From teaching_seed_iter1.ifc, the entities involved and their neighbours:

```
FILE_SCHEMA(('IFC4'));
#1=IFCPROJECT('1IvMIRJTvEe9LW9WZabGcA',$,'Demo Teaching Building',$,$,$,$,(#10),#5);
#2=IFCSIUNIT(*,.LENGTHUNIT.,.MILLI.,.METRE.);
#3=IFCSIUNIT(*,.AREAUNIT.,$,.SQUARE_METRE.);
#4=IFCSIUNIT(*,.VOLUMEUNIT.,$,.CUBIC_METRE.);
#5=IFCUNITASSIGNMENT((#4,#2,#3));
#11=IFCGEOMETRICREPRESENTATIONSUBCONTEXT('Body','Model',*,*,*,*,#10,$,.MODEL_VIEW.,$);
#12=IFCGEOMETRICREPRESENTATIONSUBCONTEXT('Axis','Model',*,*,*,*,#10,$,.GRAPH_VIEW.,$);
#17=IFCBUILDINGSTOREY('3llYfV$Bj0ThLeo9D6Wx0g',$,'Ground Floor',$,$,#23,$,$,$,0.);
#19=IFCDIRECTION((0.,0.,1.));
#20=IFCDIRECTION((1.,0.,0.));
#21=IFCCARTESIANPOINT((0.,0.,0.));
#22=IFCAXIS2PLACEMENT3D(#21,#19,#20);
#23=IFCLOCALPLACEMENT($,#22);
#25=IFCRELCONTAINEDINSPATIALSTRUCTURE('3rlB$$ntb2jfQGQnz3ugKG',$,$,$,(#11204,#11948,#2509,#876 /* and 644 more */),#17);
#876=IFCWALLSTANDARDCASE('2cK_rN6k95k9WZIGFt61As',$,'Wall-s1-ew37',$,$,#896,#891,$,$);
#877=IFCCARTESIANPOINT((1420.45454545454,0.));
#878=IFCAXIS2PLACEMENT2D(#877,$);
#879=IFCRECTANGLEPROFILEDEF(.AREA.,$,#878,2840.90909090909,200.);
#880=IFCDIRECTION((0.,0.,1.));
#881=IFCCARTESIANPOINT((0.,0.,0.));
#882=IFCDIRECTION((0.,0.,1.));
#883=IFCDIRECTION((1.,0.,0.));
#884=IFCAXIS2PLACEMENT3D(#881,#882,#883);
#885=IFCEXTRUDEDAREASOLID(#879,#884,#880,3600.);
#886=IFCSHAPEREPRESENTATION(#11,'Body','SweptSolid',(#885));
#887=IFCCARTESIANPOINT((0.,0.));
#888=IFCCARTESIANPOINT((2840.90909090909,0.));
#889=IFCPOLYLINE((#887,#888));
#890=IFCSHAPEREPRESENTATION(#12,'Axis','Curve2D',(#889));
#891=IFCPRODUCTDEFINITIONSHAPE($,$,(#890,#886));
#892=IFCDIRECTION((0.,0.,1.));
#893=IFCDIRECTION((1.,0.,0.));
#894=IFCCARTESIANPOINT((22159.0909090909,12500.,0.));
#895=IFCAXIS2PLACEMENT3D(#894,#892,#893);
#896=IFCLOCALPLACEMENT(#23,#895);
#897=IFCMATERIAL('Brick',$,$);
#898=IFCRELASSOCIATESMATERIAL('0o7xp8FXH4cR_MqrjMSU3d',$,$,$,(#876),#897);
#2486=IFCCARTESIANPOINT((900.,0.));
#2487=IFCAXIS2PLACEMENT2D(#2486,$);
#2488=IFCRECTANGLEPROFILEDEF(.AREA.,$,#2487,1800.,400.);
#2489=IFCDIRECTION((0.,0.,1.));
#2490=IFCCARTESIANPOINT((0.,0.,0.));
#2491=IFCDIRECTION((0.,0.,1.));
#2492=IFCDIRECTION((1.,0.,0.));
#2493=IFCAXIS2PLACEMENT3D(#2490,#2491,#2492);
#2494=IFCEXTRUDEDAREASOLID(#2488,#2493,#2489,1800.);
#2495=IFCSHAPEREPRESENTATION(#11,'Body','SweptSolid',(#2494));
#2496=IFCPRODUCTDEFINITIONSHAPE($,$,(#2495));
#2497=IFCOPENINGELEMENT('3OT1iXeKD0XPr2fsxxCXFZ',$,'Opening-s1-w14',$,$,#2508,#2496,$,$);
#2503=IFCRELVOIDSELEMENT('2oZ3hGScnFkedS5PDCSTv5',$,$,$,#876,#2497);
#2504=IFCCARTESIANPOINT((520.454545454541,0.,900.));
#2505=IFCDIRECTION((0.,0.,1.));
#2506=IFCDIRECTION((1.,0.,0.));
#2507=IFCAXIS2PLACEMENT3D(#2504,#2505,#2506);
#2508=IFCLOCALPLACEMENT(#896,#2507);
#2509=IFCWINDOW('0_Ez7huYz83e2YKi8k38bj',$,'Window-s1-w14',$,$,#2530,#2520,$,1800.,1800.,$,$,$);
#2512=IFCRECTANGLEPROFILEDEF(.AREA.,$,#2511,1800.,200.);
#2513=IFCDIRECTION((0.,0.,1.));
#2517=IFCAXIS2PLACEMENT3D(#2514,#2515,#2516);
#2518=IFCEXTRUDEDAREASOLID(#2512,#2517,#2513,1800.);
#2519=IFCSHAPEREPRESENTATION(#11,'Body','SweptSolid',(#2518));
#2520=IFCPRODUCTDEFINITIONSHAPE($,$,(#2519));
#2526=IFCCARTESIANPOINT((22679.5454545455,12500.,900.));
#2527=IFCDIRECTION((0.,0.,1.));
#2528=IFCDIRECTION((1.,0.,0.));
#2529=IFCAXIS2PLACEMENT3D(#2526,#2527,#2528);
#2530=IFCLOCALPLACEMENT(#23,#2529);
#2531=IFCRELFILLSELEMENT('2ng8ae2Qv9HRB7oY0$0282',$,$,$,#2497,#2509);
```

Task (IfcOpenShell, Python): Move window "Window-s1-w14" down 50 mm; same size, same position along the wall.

```python
import numpy as np
import ifcopenshell
import ifcopenshell.api.geometry
import ifcopenshell.util.placement
import ifcopenshell.util.unit

model = ifcopenshell.open("teaching_seed_iter1.ifc")
unit_scale = ifcopenshell.util.unit.calculate_unit_scale(model)

window = model.by_id(2509)
opening = window.FillsVoids[0].RelatingOpeningElement
dz = -0.05 / unit_scale

shift = np.array([0.0, 0.0, dz])
# The window is not placed relative to its opening, so move both.
for product in (opening, window):
    matrix = ifcopenshell.util.placement.get_local_placement(product.ObjectPlacement)
    matrix[:3, 3] += shift
    ifcopenshell.api.geometry.edit_object_placement(model, product=product, matrix=matrix, is_si=False)

print(f"moved by {dz * unit_scale:+.3f} m")

model.write("teaching_seed_iter1_updated.ifc")
```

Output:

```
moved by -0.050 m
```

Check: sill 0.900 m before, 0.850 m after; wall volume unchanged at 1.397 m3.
